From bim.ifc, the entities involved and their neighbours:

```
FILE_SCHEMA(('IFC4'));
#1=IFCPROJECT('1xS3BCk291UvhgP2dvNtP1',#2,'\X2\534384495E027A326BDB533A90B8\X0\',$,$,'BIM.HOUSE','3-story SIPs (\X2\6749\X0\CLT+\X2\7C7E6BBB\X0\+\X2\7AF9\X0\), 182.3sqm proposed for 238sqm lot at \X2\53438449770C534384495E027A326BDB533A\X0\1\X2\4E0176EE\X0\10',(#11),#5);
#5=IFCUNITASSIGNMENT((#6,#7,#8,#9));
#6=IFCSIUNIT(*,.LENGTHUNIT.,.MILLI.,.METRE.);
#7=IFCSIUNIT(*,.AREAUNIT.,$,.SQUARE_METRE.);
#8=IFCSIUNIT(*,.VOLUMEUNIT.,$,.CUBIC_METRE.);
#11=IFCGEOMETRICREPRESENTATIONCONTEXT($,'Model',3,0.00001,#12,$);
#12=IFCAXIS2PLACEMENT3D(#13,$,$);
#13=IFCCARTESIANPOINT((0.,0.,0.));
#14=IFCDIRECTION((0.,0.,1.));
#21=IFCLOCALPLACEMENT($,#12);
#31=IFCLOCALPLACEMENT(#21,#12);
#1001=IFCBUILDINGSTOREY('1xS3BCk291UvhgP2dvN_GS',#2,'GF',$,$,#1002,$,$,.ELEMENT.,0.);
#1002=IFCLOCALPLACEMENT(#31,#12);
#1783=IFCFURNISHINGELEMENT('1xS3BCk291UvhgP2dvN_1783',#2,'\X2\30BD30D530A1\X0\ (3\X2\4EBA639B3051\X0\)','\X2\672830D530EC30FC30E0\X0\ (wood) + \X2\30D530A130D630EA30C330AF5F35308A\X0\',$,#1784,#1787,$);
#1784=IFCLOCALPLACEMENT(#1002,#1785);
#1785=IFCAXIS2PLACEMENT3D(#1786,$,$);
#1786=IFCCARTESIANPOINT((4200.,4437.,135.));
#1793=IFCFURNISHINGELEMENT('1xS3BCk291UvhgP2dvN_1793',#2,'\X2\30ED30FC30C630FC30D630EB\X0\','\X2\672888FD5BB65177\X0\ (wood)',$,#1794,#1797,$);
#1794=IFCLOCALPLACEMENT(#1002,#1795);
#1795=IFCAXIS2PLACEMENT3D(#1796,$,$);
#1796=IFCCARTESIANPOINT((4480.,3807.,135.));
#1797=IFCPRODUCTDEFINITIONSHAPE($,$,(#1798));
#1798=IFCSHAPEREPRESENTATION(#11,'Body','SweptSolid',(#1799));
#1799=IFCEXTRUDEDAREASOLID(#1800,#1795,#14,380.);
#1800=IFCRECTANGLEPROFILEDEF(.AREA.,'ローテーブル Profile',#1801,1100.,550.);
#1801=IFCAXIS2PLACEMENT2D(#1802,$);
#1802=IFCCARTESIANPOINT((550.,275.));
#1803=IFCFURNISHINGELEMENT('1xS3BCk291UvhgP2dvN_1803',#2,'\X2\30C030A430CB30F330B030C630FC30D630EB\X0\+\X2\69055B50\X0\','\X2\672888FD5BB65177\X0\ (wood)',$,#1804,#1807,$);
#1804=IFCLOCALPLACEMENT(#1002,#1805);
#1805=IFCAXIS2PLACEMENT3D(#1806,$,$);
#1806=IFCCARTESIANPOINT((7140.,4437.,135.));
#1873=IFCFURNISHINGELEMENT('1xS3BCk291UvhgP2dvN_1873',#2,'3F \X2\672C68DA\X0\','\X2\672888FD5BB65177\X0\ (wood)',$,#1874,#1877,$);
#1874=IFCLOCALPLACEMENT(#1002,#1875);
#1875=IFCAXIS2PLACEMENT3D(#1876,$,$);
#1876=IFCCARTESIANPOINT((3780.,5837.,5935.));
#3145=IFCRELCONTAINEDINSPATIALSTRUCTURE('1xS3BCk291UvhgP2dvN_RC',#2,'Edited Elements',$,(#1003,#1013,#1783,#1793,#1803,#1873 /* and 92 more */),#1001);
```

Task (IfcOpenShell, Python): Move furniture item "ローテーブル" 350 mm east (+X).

```python
import ifcopenshell
import ifcopenshell.api.geometry
import ifcopenshell.util.placement

model = ifcopenshell.open("bim.ifc")

item = model.by_id(1793)
matrix = ifcopenshell.util.placement.get_local_placement(item.ObjectPlacement)
matrix[0, 3] += 350.0
ifcopenshell.api.geometry.edit_object_placement(model, product=item, matrix=matrix, is_si=False)

print(ifcopenshell.util.placement.get_local_placement(item.ObjectPlacement).round(3) + 0.0)

model.write("bim_edited.ifc")
```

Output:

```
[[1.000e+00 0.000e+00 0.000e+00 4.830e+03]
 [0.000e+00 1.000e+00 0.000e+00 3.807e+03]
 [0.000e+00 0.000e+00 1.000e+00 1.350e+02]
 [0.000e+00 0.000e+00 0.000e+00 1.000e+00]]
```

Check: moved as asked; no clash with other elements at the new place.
